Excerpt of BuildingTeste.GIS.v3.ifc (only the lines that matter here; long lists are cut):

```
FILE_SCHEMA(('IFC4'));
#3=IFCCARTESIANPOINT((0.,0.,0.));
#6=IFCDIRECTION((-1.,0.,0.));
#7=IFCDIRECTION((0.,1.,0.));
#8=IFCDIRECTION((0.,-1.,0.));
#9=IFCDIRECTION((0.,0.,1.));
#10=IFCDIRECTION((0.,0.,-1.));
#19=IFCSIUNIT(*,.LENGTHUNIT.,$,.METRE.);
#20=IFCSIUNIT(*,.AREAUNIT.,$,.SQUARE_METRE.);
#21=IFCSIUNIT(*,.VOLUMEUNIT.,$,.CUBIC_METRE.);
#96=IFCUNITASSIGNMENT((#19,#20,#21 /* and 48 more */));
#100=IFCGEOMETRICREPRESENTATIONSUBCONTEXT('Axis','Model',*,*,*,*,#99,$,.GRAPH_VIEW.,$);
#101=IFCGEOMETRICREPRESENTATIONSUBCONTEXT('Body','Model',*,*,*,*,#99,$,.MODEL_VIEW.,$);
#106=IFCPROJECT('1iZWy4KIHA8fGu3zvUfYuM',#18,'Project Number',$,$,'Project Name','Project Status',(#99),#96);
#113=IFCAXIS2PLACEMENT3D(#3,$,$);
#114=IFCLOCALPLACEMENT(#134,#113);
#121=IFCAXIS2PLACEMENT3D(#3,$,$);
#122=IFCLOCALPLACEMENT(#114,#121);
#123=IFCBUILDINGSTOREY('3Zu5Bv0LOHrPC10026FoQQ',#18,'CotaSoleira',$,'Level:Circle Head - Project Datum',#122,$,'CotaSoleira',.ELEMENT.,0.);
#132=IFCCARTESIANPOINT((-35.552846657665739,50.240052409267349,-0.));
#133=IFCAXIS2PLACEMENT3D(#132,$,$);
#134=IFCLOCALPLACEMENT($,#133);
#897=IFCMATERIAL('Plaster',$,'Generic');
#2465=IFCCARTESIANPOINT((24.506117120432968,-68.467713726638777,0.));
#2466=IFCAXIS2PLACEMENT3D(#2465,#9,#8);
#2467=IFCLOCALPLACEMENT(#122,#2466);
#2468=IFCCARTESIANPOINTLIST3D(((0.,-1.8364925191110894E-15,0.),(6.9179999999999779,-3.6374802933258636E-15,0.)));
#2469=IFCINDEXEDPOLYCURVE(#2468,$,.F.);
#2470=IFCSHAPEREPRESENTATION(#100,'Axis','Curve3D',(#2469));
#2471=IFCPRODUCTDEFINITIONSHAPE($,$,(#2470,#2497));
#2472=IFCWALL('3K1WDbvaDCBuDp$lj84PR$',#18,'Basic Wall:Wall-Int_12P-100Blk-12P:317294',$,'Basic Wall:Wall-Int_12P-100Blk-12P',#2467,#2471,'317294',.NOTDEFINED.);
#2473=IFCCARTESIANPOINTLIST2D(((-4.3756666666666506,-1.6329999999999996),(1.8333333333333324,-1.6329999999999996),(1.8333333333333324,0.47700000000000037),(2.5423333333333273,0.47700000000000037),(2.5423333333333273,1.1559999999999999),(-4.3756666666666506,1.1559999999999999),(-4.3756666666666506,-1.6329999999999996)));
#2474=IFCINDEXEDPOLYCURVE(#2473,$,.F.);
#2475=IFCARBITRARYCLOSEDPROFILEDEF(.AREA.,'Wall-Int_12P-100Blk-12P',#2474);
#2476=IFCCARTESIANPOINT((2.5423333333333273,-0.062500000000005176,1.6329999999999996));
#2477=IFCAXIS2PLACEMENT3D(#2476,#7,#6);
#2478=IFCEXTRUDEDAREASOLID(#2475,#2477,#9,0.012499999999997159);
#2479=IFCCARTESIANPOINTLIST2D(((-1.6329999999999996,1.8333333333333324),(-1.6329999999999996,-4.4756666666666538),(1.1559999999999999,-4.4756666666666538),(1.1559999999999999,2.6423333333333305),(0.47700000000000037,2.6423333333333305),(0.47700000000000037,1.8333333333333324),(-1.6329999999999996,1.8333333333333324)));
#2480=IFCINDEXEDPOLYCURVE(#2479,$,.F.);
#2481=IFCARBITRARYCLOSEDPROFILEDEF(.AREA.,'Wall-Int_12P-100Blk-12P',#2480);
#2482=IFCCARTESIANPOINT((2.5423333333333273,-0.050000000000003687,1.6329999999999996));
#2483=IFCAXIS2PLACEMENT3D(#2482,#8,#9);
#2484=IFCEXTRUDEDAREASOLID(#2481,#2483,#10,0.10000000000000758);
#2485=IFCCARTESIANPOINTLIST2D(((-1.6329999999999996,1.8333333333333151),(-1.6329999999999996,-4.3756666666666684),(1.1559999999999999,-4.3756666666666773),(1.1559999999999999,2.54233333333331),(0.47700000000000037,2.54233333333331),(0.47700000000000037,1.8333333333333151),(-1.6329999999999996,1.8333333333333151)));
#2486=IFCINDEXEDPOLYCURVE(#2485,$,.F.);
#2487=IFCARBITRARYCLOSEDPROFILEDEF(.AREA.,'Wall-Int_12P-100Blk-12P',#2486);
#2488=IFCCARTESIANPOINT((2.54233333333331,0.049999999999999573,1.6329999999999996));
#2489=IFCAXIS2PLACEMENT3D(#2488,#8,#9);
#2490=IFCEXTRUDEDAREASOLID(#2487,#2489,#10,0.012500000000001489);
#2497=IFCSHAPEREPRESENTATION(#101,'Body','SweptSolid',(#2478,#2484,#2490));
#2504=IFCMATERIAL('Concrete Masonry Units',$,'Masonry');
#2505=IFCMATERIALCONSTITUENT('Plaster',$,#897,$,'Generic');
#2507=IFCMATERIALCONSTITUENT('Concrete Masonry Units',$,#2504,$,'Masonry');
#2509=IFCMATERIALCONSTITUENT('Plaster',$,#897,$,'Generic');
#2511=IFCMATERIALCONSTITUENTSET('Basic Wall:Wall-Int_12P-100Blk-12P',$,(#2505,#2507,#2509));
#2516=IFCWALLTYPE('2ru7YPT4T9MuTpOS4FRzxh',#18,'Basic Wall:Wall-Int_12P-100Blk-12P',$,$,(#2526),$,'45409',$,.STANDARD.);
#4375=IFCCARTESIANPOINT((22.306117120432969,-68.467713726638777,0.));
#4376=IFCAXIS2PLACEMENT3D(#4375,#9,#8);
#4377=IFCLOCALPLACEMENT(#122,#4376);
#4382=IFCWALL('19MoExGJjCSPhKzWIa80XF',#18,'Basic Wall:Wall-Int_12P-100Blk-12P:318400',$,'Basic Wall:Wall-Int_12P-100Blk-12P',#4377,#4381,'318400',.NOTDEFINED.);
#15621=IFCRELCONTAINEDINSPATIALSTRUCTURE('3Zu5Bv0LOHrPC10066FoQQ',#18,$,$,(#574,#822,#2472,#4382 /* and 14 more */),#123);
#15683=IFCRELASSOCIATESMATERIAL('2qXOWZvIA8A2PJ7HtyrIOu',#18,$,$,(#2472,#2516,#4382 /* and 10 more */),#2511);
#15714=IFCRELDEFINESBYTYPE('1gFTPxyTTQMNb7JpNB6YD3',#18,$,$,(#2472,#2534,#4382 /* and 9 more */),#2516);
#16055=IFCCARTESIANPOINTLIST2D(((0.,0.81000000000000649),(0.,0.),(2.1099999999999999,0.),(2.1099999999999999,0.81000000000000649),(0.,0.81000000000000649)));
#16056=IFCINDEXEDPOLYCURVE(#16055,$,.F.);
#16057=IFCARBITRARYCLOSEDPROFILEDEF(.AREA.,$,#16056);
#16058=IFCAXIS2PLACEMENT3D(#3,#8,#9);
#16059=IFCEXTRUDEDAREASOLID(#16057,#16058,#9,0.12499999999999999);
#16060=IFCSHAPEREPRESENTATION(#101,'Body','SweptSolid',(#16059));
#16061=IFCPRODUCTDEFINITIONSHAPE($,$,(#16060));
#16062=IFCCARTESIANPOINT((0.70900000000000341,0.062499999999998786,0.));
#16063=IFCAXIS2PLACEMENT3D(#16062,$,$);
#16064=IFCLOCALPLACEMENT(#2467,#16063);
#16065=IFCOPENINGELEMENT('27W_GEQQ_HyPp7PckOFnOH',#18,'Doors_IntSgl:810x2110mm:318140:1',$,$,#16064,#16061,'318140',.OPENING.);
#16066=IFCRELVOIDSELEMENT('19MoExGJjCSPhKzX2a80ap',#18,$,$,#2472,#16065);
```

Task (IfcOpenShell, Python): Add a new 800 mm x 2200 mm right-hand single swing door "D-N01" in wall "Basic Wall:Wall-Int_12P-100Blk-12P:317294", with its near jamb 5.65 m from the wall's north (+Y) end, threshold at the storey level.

```python
import numpy as np
import ifcopenshell
import ifcopenshell.api.feature
import ifcopenshell.api.geometry
import ifcopenshell.api.root
import ifcopenshell.api.spatial
import ifcopenshell.geom
import ifcopenshell.util.element
import ifcopenshell.util.placement
import ifcopenshell.util.representation
import ifcopenshell.util.shape
import ifcopenshell.util.unit

model = ifcopenshell.open("BuildingTeste.GIS.v3.ifc")
unit_scale = ifcopenshell.util.unit.calculate_unit_scale(model)
settings = ifcopenshell.geom.settings()


def volume(element):
    """Net volume in cubic metres, openings subtracted."""
    shape = ifcopenshell.geom.create_shape(settings, element)
    return ifcopenshell.util.shape.get_volume(shape.geometry)


wall = model.by_guid("3K1WDbvaDCBuDp$lj84PR$")
storey = ifcopenshell.util.element.get_container(wall, ifc_class="IfcBuildingStorey")
context = ifcopenshell.util.representation.get_context(model, "Model", "Body", "MODEL_VIEW")
before = volume(wall)

width, height, from_end, sill = 0.8, 2.2, 5.65, 0.0  # metres

# The wall runs along its own X axis, and the end named is its -X end.
wall_shape = ifcopenshell.geom.create_shape(settings, wall)
x, y, z = ifcopenshell.util.shape.get_vertices(wall_shape.geometry).T
start = x.min() + from_end
face, thickness = float(y.min()), float(y.max() - y.min())
wall_matrix = ifcopenshell.util.placement.get_local_placement(wall.ObjectPlacement)
level = ifcopenshell.util.placement.get_local_placement(storey.ObjectPlacement)[2, 3]


def in_wall(x, y):
    """Placement at x, y metres in the wall's axes, at sill height."""
    matrix = wall_matrix.copy()
    matrix[:, 3] = wall_matrix @ np.array([x / unit_scale, y / unit_scale, 0.0, 1.0])
    matrix[2, 3] = level + sill / unit_scale
    return matrix


# Opening: a box that overshoots both wall faces by 50 mm.
opening = ifcopenshell.api.root.create_entity(model, ifc_class="IfcOpeningElement", predefined_type="OPENING")
box = ifcopenshell.api.geometry.add_wall_representation(
    model, context=context, length=width, height=height, thickness=thickness + 0.1
)
ifcopenshell.api.geometry.assign_representation(model, product=opening, representation=box)
ifcopenshell.api.geometry.edit_object_placement(model, product=opening, matrix=in_wall(start, face - 0.05), is_si=False)
ifcopenshell.api.feature.add_feature(model, feature=opening, element=wall)

door = ifcopenshell.api.root.create_entity(model, ifc_class="IfcDoor", name="D-N01", predefined_type="DOOR")
door.OverallWidth, door.OverallHeight = width / unit_scale, height / unit_scale
door.OperationType = "SINGLE_SWING_RIGHT"
body = ifcopenshell.api.geometry.add_door_representation(
    model,
    context=context,
    overall_width=door.OverallWidth,
    overall_height=door.OverallHeight,
    operation_type="SINGLE_SWING_RIGHT",
    lining_properties={"LiningDepth": thickness / unit_scale, "ThresholdDepth": thickness / unit_scale},
)
ifcopenshell.api.geometry.assign_representation(model, product=door, representation=body)
ifcopenshell.api.spatial.assign_container(model, products=[door], relating_structure=storey)
ifcopenshell.api.feature.add_filling(model, opening=opening, element=door)

# The lining spans the wall, so the door starts at the wall face.
ifcopenshell.api.geometry.edit_object_placement(model, product=door, matrix=in_wall(start, face), is_si=False)

after = volume(wall)

print(f"wall volume {before:.3f} -> {after:.3f} m3")

model.write("BuildingTeste.GIS.v3_updated.ifc")
```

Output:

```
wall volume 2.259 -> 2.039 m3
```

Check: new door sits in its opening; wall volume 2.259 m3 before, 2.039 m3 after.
